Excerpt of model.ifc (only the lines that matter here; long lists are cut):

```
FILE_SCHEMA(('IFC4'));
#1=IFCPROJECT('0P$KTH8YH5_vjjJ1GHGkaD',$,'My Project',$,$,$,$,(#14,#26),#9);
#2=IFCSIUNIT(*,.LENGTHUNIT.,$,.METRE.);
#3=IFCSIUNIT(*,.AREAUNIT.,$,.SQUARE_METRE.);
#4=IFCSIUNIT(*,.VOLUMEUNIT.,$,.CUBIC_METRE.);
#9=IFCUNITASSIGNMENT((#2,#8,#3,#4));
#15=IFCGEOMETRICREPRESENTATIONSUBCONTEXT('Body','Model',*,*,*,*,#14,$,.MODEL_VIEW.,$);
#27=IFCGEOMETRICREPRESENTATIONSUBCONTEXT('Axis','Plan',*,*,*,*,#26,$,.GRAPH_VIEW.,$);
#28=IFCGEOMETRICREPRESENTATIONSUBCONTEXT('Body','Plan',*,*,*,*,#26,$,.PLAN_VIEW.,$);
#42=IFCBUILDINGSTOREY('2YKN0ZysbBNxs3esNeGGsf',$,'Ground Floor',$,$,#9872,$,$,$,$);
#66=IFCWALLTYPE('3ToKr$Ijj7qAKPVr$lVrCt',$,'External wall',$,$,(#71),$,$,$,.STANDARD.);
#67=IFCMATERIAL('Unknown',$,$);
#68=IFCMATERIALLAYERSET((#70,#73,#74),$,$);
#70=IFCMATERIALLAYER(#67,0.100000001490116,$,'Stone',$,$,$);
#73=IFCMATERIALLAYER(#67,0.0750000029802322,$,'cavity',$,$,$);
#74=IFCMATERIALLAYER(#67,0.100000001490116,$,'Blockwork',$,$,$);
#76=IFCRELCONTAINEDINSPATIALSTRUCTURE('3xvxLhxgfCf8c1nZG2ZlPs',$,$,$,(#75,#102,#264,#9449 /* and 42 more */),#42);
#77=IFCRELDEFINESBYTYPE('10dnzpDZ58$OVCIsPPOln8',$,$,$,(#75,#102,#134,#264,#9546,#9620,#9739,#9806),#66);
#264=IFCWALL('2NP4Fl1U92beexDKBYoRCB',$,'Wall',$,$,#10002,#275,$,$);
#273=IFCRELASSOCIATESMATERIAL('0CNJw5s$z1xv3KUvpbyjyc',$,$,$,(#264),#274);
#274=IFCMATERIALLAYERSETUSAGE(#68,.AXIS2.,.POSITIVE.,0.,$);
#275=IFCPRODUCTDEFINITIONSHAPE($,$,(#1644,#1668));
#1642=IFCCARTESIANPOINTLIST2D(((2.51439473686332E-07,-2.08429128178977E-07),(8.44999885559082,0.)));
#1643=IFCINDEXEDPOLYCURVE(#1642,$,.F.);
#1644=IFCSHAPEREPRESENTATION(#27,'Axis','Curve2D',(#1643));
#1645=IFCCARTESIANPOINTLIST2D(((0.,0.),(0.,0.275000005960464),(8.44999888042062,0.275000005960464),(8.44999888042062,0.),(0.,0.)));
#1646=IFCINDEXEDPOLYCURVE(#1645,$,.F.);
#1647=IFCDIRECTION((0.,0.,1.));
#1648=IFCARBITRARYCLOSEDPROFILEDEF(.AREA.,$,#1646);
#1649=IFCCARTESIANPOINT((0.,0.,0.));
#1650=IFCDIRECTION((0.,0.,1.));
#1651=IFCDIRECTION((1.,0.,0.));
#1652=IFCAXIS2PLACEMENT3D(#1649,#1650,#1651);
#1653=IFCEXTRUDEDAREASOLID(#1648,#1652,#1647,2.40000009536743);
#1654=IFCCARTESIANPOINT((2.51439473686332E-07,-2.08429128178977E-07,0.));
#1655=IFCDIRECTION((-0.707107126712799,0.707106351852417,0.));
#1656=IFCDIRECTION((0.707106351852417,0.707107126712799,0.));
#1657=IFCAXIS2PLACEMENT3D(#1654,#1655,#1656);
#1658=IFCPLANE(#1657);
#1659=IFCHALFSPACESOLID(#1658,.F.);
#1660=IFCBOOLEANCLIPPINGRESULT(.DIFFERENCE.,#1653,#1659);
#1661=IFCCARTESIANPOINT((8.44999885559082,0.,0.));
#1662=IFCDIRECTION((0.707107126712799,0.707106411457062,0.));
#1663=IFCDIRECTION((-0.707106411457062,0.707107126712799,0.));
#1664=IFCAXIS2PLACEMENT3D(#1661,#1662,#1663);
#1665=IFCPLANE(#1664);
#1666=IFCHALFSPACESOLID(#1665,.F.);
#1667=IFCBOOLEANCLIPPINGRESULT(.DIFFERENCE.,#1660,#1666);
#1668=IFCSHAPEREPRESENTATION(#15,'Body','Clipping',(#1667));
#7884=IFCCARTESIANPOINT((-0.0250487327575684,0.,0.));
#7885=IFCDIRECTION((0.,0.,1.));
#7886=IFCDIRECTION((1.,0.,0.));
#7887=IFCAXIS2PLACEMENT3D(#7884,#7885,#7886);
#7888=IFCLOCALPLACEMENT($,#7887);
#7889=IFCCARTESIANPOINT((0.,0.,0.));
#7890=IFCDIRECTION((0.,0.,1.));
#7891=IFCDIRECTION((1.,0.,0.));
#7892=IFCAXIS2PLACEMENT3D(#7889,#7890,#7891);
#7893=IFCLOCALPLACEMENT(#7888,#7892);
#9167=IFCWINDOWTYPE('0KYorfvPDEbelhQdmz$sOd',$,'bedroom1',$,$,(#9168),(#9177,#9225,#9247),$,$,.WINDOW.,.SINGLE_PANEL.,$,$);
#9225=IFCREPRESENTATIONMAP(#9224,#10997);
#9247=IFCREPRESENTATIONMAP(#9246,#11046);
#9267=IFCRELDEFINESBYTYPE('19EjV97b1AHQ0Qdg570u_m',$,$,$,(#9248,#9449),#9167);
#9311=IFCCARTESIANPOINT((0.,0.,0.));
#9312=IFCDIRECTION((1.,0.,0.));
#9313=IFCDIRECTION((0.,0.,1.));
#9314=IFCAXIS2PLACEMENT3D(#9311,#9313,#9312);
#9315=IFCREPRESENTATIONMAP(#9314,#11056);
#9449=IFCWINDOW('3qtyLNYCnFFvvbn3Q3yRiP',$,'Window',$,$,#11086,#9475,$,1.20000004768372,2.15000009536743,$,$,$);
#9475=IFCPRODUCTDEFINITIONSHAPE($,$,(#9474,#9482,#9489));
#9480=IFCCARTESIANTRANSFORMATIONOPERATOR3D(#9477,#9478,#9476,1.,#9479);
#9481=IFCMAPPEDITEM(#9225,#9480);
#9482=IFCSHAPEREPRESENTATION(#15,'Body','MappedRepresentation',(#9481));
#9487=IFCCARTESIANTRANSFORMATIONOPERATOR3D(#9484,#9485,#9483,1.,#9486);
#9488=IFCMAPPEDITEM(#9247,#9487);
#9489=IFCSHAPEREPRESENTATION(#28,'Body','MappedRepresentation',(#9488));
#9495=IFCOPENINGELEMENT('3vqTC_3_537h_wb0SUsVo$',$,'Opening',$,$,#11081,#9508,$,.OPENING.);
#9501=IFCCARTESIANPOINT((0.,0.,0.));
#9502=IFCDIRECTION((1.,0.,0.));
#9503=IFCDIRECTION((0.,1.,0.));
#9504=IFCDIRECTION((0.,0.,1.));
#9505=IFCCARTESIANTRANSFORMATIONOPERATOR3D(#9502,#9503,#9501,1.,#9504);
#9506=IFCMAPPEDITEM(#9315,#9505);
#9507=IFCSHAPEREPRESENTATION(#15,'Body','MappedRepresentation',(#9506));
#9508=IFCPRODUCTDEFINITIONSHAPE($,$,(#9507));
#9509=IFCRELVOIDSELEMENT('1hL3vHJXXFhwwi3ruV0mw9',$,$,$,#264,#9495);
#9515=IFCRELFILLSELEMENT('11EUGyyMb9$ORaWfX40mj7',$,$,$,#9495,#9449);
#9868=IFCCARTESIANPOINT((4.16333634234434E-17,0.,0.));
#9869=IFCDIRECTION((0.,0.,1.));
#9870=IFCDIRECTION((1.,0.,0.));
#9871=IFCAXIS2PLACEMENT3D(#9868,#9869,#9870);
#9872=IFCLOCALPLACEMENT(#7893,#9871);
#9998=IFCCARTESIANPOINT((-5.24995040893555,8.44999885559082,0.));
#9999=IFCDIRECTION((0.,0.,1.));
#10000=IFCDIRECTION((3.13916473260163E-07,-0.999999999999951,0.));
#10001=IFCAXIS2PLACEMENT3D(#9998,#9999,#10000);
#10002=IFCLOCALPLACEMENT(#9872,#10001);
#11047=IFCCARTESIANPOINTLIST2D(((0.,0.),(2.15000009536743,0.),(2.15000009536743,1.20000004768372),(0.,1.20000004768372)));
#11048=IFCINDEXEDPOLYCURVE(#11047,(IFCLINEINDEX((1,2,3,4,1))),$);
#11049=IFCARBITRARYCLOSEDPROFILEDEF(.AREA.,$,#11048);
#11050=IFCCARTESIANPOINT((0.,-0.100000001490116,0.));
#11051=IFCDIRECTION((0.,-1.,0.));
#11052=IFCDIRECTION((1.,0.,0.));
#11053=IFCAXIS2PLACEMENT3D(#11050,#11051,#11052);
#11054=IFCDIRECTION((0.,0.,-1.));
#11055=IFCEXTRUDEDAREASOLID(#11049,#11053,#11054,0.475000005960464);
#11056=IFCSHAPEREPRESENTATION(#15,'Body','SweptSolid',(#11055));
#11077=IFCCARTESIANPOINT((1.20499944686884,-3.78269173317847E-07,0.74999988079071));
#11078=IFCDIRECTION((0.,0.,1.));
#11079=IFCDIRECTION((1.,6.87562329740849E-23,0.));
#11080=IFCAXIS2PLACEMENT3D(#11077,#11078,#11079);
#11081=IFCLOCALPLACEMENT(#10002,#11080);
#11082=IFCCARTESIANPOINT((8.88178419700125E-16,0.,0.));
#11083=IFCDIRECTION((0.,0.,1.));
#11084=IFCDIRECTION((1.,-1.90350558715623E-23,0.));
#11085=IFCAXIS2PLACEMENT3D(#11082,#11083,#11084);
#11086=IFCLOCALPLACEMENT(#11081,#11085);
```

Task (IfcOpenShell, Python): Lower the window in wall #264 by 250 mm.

```python
import numpy as np
import ifcopenshell
import ifcopenshell.api.geometry
import ifcopenshell.util.placement
import ifcopenshell.util.unit

model = ifcopenshell.open("model.ifc")
unit_scale = ifcopenshell.util.unit.calculate_unit_scale(model)

window = model.by_guid("3qtyLNYCnFFvvbn3Q3yRiP")
opening = window.FillsVoids[0].RelatingOpeningElement
dz = -0.25

shift = np.array([0.0, 0.0, dz])
# The window is placed relative to its opening, so it follows when the opening moves.
matrix = ifcopenshell.util.placement.get_local_placement(opening.ObjectPlacement)
matrix[:3, 3] += shift
ifcopenshell.api.geometry.edit_object_placement(
    model, product=opening, matrix=matrix, is_si=False, should_transform_children=True
)

print(f"moved by {dz * unit_scale:+.3f} m")

model.write("model_edited.ifc")
```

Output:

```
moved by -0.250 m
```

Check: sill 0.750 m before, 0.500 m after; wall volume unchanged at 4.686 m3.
